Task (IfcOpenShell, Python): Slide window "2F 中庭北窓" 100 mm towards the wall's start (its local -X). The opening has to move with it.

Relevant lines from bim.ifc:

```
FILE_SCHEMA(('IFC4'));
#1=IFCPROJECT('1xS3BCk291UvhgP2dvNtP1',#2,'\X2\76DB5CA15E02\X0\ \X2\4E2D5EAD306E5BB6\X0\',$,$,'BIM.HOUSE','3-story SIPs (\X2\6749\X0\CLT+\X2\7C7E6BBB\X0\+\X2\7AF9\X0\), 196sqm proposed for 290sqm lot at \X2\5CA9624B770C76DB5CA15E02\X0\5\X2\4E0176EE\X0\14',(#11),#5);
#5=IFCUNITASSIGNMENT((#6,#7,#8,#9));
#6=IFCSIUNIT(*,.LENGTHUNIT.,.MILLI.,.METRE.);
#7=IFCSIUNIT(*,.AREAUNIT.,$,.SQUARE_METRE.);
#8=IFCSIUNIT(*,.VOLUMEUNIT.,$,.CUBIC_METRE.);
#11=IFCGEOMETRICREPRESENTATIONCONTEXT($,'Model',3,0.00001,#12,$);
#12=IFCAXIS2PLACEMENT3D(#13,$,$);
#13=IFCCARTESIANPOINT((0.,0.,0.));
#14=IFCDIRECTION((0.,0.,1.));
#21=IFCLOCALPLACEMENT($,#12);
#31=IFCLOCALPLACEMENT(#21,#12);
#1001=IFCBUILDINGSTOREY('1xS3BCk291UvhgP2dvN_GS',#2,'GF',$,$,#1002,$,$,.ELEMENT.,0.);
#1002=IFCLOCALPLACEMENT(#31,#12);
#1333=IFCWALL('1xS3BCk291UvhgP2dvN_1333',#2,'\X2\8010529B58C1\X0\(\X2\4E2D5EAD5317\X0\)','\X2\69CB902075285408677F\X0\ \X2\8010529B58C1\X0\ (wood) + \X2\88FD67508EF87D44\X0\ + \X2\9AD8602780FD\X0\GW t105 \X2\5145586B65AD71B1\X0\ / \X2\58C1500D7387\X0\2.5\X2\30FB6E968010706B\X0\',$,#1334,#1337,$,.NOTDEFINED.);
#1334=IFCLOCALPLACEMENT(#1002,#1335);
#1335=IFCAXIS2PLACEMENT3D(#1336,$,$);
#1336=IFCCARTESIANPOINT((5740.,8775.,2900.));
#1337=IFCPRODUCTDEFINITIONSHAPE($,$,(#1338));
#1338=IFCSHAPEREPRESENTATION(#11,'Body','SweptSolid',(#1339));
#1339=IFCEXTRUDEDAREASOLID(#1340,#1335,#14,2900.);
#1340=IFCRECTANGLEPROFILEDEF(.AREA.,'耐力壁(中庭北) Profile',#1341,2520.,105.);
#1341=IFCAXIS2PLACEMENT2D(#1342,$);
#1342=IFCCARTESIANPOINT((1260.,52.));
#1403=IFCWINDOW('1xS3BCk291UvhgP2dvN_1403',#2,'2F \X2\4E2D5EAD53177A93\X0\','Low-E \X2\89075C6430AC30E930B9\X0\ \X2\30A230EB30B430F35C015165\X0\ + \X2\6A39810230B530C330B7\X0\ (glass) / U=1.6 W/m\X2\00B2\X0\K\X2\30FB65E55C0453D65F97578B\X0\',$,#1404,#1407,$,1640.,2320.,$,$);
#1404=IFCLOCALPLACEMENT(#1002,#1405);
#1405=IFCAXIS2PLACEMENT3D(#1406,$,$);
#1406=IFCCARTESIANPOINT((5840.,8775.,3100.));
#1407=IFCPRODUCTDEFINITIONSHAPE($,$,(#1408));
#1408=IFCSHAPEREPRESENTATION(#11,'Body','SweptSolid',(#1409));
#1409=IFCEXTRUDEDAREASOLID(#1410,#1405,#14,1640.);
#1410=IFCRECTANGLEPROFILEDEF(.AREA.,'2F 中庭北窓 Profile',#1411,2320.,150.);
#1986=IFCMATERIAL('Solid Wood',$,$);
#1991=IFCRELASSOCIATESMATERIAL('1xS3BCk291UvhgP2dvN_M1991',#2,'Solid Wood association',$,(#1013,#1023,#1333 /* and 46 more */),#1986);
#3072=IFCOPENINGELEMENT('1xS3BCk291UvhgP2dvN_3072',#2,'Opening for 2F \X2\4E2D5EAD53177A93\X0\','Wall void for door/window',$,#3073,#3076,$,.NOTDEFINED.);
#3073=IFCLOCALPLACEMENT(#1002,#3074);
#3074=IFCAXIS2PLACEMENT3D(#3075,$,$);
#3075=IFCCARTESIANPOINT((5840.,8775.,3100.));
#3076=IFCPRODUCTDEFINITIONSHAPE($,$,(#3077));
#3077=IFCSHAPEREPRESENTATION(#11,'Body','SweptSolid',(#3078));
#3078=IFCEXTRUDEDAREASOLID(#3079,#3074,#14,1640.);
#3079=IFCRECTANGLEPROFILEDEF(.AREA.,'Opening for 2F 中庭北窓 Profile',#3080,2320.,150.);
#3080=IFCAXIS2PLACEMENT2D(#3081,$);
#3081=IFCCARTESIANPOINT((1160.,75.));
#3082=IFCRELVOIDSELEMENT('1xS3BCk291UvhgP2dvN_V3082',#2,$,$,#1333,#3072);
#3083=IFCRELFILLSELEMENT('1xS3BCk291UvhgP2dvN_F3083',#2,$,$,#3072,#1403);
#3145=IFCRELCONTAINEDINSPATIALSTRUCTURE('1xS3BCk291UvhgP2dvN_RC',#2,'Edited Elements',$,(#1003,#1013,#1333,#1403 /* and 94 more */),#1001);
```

```python
import ifcopenshell
import ifcopenshell.api.geometry
import ifcopenshell.util.placement
import ifcopenshell.util.unit

model = ifcopenshell.open("bim.ifc")
unit_scale = ifcopenshell.util.unit.calculate_unit_scale(model)

window = model.by_id(1403)
opening = window.FillsVoids[0].RelatingOpeningElement
wall = opening.VoidsElements[0].RelatingBuildingElement

wall_matrix = ifcopenshell.util.placement.get_local_placement(wall.ObjectPlacement)
shift = wall_matrix[:3, 0] * -0.1 / unit_scale
before = ifcopenshell.util.placement.get_local_placement(window.ObjectPlacement)[:3, 3].copy()

# The window is not placed relative to its opening, so move both.
for product in (opening, window):
    matrix = ifcopenshell.util.placement.get_local_placement(product.ObjectPlacement)
    matrix[:3, 3] += shift
    ifcopenshell.api.geometry.edit_object_placement(model, product=product, matrix=matrix, is_si=False)

after = ifcopenshell.util.placement.get_local_placement(window.ObjectPlacement)[:3, 3]
print("window moved by", (after - before).round(3) + 0.0)

model.write("bim_edited.ifc")
```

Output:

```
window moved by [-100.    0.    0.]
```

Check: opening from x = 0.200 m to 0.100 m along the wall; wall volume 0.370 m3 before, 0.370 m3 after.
